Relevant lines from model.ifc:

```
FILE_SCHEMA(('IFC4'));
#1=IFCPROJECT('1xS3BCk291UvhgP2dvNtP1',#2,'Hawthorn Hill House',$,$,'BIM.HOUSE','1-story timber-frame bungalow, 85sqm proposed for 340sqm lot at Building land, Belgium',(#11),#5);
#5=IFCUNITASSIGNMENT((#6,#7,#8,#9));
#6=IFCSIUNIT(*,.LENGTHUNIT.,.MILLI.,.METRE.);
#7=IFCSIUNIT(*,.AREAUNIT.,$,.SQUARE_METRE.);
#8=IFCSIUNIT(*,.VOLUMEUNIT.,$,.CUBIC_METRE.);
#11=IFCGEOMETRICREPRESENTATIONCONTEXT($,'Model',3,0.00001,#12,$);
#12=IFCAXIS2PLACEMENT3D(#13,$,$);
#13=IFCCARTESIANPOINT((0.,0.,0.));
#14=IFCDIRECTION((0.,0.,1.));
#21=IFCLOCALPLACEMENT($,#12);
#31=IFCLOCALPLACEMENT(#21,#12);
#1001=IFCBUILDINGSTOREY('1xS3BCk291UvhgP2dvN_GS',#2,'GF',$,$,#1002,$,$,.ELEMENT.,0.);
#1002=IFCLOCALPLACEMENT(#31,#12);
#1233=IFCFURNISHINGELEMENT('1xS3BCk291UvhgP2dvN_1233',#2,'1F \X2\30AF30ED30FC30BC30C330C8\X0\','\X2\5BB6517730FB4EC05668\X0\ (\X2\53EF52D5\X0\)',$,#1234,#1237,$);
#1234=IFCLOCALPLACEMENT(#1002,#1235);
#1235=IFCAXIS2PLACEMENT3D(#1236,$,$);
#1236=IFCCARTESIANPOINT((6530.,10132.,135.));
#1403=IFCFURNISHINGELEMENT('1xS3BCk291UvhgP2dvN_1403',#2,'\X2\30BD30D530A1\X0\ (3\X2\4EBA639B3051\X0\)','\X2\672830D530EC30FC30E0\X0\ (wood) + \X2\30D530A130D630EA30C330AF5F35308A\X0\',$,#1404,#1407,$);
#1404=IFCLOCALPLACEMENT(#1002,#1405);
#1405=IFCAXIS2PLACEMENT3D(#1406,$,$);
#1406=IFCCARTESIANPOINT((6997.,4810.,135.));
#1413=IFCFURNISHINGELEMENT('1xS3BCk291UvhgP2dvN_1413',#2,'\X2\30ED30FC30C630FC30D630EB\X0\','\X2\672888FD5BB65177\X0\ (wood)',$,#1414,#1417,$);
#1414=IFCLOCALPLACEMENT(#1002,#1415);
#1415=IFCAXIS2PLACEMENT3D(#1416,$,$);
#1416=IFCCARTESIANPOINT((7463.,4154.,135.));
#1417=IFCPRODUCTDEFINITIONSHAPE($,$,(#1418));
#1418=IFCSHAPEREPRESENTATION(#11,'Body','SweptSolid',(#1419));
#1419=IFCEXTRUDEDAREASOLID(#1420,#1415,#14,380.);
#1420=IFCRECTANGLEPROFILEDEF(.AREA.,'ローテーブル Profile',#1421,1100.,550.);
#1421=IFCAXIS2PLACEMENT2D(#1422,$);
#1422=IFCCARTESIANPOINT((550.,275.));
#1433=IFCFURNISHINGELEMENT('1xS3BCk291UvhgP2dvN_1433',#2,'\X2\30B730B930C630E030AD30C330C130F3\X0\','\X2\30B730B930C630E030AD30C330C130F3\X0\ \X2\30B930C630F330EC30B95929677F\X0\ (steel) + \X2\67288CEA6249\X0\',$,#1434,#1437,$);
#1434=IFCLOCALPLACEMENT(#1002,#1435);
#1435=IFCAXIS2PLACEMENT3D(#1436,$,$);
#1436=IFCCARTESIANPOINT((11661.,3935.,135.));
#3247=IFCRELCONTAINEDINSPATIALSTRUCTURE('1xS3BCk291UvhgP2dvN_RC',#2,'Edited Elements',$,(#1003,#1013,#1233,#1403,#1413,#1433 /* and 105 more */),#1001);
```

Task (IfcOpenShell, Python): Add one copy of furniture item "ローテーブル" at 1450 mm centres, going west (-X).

```python
import numpy as np
import ifcopenshell
import ifcopenshell.api.geometry
import ifcopenshell.api.root
import ifcopenshell.util.element
import ifcopenshell.util.placement
import ifcopenshell.util.unit

model = ifcopenshell.open("model.ifc")
unit_scale = ifcopenshell.util.unit.calculate_unit_scale(model)


def reuse_history(source, copy):
    """copy_class also copies each property set's owner history, people and application; keep the originals."""
    for rel in copy.IsDefinedBy:
        if rel.is_a("IfcRelDefinesByProperties") and (history := rel.RelatingPropertyDefinition.OwnerHistory):
            rel.RelatingPropertyDefinition.OwnerHistory = source.OwnerHistory
            ifcopenshell.util.element.remove_deep2(model, history)


source = model.by_guid("1xS3BCk291UvhgP2dvN_1413")
base = ifcopenshell.util.placement.get_local_placement(source.ObjectPlacement)
step = np.array([-1.0, 0.0, 0.0]) * 1.45 / unit_scale

for i in range(1, 2):
    copy = ifcopenshell.api.root.copy_class(model, product=source)
    copy.Representation = ifcopenshell.util.element.copy_deep(
        model, source.Representation, exclude=["IfcGeometricRepresentationContext", "IfcRepresentationMap"]
    )
    reuse_history(source, copy)
    matrix = base.copy()
    matrix[:3, 3] += i * step
    print("added at", matrix[:3, 3].round(3) + 0.0)
    ifcopenshell.api.geometry.edit_object_placement(model, product=copy, matrix=matrix, is_si=False)

model.write("model_updated.ifc")
```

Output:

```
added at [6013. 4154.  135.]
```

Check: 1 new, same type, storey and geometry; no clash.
